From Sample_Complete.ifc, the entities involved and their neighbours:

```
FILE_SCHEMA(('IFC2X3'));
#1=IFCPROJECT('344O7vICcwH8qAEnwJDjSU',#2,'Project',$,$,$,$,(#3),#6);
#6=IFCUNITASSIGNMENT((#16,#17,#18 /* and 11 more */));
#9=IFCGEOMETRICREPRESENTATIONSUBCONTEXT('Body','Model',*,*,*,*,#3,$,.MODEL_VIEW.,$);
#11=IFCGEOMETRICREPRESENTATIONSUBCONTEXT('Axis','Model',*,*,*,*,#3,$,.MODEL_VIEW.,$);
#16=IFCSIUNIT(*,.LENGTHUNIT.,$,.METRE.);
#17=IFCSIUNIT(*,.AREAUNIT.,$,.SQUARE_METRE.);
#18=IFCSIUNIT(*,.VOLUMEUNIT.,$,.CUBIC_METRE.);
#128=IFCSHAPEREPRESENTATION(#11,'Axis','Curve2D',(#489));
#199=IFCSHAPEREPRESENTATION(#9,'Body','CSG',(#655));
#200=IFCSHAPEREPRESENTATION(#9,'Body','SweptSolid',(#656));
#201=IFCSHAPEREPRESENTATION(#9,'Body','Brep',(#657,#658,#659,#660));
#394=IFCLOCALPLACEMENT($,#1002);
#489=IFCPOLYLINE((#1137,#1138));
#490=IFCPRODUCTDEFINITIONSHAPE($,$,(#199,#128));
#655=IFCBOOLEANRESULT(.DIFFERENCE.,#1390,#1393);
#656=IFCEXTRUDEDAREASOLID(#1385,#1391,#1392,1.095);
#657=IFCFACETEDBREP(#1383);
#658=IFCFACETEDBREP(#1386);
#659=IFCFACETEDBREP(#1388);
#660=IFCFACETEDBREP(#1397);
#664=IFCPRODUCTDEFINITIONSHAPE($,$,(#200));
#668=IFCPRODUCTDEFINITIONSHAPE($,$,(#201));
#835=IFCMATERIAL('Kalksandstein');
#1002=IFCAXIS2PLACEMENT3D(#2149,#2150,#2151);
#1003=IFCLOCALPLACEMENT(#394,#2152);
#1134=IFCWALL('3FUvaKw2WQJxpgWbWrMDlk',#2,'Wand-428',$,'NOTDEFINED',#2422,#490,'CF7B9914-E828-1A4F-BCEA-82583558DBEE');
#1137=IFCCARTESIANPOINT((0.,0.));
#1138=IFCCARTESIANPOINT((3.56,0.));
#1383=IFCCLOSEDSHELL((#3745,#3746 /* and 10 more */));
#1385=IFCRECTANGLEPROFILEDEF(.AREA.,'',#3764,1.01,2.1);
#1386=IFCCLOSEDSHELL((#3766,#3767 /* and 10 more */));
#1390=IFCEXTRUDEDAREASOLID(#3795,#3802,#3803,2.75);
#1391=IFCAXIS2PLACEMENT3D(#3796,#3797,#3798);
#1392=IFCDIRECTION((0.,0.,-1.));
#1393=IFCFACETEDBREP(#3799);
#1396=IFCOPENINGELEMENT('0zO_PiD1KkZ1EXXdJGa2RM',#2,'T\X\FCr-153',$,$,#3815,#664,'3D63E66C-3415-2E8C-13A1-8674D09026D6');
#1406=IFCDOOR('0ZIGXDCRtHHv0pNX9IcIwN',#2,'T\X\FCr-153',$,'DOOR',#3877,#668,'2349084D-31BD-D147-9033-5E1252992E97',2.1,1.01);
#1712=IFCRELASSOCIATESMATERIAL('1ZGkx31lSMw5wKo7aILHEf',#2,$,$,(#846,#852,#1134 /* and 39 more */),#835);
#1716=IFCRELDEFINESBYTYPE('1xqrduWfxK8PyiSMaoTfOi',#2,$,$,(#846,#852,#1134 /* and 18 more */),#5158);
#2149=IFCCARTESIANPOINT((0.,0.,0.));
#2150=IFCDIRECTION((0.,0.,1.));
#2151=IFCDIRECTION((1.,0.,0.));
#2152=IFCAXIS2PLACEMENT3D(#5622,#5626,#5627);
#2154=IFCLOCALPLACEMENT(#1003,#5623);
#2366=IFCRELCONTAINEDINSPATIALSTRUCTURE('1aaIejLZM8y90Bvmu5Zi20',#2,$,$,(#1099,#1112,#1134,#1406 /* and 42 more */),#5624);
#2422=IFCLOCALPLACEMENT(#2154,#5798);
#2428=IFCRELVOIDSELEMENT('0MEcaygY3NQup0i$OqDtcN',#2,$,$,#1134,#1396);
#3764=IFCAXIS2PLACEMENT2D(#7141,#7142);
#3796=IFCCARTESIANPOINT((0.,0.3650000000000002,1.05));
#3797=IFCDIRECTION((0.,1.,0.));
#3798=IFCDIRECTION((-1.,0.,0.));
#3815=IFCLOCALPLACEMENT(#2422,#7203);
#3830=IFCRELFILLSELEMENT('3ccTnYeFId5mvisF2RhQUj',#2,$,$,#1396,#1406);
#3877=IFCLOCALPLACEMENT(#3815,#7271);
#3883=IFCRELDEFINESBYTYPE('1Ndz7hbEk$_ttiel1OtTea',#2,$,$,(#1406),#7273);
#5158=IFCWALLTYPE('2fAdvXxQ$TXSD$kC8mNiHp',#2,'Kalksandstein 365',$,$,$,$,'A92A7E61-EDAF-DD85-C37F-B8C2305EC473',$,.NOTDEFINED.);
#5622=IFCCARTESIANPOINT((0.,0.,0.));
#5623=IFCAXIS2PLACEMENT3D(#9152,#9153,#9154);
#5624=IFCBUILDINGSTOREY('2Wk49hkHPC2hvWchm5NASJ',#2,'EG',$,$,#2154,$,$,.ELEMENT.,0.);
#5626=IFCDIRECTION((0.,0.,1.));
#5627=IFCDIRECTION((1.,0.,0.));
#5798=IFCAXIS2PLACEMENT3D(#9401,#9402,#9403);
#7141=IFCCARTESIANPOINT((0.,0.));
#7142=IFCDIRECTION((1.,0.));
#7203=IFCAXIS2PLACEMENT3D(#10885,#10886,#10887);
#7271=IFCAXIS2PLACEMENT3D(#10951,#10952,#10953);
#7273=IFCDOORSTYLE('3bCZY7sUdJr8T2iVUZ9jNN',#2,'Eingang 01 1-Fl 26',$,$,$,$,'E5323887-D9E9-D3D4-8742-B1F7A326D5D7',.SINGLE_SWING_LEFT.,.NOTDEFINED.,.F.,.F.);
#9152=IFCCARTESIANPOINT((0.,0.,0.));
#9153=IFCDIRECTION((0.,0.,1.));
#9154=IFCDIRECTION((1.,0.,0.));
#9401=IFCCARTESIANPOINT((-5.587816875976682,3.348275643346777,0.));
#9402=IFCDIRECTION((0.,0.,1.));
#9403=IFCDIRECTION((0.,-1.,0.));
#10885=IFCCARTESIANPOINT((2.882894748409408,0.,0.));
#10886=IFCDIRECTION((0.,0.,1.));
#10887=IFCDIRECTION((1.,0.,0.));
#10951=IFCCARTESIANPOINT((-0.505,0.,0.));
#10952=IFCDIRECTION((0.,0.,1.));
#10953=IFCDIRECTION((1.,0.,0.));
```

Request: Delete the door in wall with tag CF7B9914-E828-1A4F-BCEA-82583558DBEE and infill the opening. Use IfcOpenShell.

```python
import ifcopenshell
import ifcopenshell.api.feature
import ifcopenshell.api.root
import ifcopenshell.geom
import ifcopenshell.util.shape

model = ifcopenshell.open("Sample_Complete.ifc")
settings = ifcopenshell.geom.settings()


def volume(element):
    """Net volume in cubic metres, openings subtracted."""
    shape = ifcopenshell.geom.create_shape(settings, element)
    return ifcopenshell.util.shape.get_volume(shape.geometry)


door = model.by_guid("0ZIGXDCRtHHv0pNX9IcIwN")
opening = door.FillsVoids[0].RelatingOpeningElement
wall = opening.VoidsElements[0].RelatingBuildingElement
before = volume(wall)

ifcopenshell.api.root.remove_product(model, product=door)
ifcopenshell.api.feature.remove_feature(model, feature=opening)

after = volume(wall)

print(f"wall volume {before:.3f} -> {after:.3f} m3")

model.write("Sample_Complete-out.ifc")
```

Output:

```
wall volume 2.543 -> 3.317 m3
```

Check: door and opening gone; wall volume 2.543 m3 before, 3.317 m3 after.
